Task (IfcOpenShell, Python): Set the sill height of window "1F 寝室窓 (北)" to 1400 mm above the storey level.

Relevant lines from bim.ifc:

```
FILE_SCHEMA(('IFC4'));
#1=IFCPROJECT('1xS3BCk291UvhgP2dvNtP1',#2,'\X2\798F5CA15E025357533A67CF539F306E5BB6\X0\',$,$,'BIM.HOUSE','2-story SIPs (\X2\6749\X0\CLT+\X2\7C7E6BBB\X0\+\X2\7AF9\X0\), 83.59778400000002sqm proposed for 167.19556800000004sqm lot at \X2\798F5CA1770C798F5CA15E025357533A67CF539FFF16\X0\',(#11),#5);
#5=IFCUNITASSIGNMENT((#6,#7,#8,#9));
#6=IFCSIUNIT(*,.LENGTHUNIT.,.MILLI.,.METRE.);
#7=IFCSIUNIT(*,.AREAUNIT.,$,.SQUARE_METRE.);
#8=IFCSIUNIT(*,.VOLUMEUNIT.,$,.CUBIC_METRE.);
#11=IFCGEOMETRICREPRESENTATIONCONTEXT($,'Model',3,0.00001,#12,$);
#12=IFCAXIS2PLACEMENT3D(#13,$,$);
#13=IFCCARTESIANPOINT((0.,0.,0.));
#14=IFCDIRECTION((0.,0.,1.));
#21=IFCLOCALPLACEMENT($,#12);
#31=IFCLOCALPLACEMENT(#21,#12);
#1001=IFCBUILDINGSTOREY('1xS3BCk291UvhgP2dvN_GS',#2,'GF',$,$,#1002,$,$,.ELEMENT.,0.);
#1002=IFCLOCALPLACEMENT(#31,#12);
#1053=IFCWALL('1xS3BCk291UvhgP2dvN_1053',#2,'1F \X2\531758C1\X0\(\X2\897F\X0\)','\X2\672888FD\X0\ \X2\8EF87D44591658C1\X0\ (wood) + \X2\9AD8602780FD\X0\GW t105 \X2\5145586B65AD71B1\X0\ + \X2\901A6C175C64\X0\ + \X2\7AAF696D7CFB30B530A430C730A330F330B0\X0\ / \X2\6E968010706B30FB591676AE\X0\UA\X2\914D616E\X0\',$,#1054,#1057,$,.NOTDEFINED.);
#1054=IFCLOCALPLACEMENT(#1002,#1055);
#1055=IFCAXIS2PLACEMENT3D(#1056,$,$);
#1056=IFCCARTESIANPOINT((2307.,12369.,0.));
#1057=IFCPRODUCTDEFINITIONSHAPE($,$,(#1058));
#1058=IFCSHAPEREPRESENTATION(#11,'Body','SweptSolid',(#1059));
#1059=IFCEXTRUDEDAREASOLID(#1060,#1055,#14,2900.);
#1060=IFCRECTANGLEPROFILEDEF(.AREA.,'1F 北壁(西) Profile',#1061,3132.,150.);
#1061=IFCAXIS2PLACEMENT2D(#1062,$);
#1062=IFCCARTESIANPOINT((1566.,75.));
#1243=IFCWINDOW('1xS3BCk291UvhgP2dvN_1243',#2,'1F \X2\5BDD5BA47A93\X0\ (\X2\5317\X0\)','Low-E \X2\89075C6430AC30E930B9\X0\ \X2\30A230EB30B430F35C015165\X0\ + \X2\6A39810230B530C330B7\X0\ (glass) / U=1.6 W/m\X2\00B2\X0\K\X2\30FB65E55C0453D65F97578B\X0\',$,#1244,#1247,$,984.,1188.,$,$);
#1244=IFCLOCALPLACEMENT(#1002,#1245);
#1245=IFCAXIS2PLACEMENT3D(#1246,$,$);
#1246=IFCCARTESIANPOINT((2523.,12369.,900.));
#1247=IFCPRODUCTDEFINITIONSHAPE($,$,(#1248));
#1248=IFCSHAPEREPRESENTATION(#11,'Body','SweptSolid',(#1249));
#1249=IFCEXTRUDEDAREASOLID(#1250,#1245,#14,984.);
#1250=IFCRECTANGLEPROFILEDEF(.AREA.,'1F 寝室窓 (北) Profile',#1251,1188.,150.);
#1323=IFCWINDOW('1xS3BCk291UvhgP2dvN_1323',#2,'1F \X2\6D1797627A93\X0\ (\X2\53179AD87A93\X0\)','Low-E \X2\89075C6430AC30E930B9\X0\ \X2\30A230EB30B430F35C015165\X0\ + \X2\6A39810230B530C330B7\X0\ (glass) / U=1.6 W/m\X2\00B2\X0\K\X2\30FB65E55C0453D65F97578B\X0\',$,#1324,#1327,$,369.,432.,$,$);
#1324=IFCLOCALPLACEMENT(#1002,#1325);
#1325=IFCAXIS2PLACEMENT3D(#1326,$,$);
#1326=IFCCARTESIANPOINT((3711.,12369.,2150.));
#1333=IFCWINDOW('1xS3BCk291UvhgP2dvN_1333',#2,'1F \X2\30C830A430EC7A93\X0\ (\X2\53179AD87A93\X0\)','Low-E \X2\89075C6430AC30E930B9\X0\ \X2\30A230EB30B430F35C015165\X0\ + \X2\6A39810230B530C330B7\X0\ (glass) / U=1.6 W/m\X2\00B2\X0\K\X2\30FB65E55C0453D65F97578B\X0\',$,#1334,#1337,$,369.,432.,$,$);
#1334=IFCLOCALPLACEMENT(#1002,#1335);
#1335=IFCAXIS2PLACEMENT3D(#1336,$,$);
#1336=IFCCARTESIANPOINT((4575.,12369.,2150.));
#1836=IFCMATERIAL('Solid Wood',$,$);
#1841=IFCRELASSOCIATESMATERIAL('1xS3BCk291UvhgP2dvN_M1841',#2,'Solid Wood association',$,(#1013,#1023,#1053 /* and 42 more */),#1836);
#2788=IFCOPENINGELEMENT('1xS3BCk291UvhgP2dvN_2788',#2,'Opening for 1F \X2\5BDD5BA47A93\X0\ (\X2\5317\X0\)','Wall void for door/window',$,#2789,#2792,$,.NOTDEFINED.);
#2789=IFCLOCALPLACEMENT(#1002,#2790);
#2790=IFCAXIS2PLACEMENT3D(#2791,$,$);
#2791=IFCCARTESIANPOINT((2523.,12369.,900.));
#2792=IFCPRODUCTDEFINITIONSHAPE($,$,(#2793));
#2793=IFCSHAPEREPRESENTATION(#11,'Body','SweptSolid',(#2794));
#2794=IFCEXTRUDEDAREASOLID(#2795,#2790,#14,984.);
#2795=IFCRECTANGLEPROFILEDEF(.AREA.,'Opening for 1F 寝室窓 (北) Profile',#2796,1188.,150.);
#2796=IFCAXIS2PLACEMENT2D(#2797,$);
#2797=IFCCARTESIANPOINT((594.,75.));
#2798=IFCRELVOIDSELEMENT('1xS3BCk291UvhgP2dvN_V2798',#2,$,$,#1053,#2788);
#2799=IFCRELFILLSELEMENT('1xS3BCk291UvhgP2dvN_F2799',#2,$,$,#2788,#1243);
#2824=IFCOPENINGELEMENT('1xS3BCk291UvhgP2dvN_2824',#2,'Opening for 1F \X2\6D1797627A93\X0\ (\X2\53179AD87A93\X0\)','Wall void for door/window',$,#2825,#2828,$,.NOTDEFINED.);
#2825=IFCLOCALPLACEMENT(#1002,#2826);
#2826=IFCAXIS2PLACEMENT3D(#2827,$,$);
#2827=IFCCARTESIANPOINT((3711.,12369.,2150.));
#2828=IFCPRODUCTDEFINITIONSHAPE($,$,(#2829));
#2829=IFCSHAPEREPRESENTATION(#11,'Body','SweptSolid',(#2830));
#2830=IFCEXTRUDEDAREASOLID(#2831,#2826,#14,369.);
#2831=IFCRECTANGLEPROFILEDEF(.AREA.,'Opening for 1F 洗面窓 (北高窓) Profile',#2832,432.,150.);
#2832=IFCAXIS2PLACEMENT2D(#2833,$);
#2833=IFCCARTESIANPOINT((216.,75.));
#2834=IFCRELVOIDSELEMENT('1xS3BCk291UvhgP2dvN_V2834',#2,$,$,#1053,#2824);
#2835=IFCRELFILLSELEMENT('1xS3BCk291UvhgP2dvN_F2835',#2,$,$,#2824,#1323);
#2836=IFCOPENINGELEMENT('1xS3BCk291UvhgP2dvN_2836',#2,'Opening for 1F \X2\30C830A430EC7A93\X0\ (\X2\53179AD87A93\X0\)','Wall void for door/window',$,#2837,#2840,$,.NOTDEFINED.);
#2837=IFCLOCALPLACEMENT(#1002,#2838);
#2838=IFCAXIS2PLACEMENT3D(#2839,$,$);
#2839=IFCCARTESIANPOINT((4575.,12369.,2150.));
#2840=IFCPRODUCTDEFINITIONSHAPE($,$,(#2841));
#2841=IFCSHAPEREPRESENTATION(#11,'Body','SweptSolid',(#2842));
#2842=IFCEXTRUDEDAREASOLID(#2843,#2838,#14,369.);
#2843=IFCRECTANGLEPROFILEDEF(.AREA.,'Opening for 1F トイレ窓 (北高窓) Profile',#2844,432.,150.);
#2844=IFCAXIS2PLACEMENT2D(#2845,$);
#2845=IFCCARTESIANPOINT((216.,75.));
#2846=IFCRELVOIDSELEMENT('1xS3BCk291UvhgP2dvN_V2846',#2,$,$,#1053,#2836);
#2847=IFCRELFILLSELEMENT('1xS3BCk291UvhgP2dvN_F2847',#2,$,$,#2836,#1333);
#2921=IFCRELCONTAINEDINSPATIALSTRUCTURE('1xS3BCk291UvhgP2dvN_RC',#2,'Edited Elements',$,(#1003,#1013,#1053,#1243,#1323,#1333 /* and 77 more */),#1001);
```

```python
import numpy as np
import ifcopenshell
import ifcopenshell.api.geometry
import ifcopenshell.geom
import ifcopenshell.util.element
import ifcopenshell.util.placement
import ifcopenshell.util.shape
import ifcopenshell.util.unit

model = ifcopenshell.open("bim.ifc")
unit_scale = ifcopenshell.util.unit.calculate_unit_scale(model)

window = model.by_guid("1xS3BCk291UvhgP2dvN_1243")
opening = window.FillsVoids[0].RelatingOpeningElement
storey = ifcopenshell.util.element.get_container(window, ifc_class="IfcBuildingStorey")
level = ifcopenshell.util.placement.get_local_placement(storey.ObjectPlacement)[2, 3]

# The opening's origin need not be at the sill, so measure its lowest point.
shape = ifcopenshell.geom.create_shape(ifcopenshell.geom.settings(), opening)
bottom = ifcopenshell.util.shape.get_shape_bottom_elevation(shape, shape.geometry) / unit_scale
dz = level + 1.4 / unit_scale - bottom

shift = np.array([0.0, 0.0, dz])
# The window is not placed relative to its opening, so move both.
for product in (opening, window):
    matrix = ifcopenshell.util.placement.get_local_placement(product.ObjectPlacement)
    matrix[:3, 3] += shift
    ifcopenshell.api.geometry.edit_object_placement(model, product=product, matrix=matrix, is_si=False)

print(f"moved by {dz * unit_scale:+.3f} m")

model.write("bim_updated.ifc")
```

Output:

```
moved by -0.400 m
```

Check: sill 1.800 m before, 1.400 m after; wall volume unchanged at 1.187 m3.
